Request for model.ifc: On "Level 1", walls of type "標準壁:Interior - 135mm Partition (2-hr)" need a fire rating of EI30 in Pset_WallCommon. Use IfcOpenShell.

First a look at what the model holds.

```python
import ifcopenshell
import ifcopenshell.util.element

model = ifcopenshell.open("model.ifc")
print(model.schema)
storey = next(s for s in model.by_type("IfcBuildingStorey") if s.Name == "Level 1")
walls = [e for e in ifcopenshell.util.element.get_decomposition(storey) if e.is_a("IfcWall")]
seen = {}
for e in walls:
    element_type = ifcopenshell.util.element.get_type(e)
    key = (element_type.Name if element_type != e and element_type else None, ifcopenshell.util.element.get_pset(e, "Pset_WallCommon", "FireRating"))
    seen[key] = seen.get(key, 0) + 1
for (name, value), count in sorted(seen.items(), key=str):
    print(count, "x", name, "|", value)
```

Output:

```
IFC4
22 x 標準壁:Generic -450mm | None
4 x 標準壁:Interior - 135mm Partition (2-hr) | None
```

```python
import ifcopenshell
import ifcopenshell.api.pset
import ifcopenshell.util.element

model = ifcopenshell.open("model.ifc")

storey = next(s for s in model.by_type("IfcBuildingStorey") if s.Name == "Level 1")
walls = [e for e in ifcopenshell.util.element.get_decomposition(storey) if e.is_a("IfcWall")]

count = 0
for e in walls:
    element_type = ifcopenshell.util.element.get_type(e)
    if element_type in (None, e) or element_type.Name != "標準壁:Interior - 135mm Partition (2-hr)":
        continue
    # add_pset returns the element's existing set when there is one.
    pset = ifcopenshell.api.pset.add_pset(model, product=e, name="Pset_WallCommon")
    ifcopenshell.api.pset.edit_pset(model, pset=pset, properties={"FireRating": "EI30"})
    count += 1

print(count, "walls updated")

model.write("model_edited.ifc")
```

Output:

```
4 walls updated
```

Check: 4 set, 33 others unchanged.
